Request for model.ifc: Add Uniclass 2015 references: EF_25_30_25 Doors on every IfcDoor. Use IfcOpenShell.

First a look at what the model holds.

```python
import ifcopenshell

model = ifcopenshell.open("model.ifc")
print(model.schema)
print("classifications:", [c.Name for c in model.by_type("IfcClassification")])
for ifc_class in ("IfcDoor", "IfcRoof", "IfcStair", "IfcWall", "IfcWindow"):
    print(ifc_class, len(model.by_type(ifc_class)))
```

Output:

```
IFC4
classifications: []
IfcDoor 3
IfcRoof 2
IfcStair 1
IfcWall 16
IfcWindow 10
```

```python
import ifcopenshell
import ifcopenshell.api.classification

model = ifcopenshell.open("model.ifc")

system = ifcopenshell.api.classification.add_classification(model, classification="Uniclass 2015")

codes = {
    "IfcDoor": ("EF_25_30_25", "Doors"),
}
for ifc_class, (code, name) in codes.items():
    products = model.by_type(ifc_class)
    ifcopenshell.api.classification.add_reference(
        model, products=products, classification=system, identification=code, name=name
    )
    print(code, len(products))

model.write("model_rev.ifc")
```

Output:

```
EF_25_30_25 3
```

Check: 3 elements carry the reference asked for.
